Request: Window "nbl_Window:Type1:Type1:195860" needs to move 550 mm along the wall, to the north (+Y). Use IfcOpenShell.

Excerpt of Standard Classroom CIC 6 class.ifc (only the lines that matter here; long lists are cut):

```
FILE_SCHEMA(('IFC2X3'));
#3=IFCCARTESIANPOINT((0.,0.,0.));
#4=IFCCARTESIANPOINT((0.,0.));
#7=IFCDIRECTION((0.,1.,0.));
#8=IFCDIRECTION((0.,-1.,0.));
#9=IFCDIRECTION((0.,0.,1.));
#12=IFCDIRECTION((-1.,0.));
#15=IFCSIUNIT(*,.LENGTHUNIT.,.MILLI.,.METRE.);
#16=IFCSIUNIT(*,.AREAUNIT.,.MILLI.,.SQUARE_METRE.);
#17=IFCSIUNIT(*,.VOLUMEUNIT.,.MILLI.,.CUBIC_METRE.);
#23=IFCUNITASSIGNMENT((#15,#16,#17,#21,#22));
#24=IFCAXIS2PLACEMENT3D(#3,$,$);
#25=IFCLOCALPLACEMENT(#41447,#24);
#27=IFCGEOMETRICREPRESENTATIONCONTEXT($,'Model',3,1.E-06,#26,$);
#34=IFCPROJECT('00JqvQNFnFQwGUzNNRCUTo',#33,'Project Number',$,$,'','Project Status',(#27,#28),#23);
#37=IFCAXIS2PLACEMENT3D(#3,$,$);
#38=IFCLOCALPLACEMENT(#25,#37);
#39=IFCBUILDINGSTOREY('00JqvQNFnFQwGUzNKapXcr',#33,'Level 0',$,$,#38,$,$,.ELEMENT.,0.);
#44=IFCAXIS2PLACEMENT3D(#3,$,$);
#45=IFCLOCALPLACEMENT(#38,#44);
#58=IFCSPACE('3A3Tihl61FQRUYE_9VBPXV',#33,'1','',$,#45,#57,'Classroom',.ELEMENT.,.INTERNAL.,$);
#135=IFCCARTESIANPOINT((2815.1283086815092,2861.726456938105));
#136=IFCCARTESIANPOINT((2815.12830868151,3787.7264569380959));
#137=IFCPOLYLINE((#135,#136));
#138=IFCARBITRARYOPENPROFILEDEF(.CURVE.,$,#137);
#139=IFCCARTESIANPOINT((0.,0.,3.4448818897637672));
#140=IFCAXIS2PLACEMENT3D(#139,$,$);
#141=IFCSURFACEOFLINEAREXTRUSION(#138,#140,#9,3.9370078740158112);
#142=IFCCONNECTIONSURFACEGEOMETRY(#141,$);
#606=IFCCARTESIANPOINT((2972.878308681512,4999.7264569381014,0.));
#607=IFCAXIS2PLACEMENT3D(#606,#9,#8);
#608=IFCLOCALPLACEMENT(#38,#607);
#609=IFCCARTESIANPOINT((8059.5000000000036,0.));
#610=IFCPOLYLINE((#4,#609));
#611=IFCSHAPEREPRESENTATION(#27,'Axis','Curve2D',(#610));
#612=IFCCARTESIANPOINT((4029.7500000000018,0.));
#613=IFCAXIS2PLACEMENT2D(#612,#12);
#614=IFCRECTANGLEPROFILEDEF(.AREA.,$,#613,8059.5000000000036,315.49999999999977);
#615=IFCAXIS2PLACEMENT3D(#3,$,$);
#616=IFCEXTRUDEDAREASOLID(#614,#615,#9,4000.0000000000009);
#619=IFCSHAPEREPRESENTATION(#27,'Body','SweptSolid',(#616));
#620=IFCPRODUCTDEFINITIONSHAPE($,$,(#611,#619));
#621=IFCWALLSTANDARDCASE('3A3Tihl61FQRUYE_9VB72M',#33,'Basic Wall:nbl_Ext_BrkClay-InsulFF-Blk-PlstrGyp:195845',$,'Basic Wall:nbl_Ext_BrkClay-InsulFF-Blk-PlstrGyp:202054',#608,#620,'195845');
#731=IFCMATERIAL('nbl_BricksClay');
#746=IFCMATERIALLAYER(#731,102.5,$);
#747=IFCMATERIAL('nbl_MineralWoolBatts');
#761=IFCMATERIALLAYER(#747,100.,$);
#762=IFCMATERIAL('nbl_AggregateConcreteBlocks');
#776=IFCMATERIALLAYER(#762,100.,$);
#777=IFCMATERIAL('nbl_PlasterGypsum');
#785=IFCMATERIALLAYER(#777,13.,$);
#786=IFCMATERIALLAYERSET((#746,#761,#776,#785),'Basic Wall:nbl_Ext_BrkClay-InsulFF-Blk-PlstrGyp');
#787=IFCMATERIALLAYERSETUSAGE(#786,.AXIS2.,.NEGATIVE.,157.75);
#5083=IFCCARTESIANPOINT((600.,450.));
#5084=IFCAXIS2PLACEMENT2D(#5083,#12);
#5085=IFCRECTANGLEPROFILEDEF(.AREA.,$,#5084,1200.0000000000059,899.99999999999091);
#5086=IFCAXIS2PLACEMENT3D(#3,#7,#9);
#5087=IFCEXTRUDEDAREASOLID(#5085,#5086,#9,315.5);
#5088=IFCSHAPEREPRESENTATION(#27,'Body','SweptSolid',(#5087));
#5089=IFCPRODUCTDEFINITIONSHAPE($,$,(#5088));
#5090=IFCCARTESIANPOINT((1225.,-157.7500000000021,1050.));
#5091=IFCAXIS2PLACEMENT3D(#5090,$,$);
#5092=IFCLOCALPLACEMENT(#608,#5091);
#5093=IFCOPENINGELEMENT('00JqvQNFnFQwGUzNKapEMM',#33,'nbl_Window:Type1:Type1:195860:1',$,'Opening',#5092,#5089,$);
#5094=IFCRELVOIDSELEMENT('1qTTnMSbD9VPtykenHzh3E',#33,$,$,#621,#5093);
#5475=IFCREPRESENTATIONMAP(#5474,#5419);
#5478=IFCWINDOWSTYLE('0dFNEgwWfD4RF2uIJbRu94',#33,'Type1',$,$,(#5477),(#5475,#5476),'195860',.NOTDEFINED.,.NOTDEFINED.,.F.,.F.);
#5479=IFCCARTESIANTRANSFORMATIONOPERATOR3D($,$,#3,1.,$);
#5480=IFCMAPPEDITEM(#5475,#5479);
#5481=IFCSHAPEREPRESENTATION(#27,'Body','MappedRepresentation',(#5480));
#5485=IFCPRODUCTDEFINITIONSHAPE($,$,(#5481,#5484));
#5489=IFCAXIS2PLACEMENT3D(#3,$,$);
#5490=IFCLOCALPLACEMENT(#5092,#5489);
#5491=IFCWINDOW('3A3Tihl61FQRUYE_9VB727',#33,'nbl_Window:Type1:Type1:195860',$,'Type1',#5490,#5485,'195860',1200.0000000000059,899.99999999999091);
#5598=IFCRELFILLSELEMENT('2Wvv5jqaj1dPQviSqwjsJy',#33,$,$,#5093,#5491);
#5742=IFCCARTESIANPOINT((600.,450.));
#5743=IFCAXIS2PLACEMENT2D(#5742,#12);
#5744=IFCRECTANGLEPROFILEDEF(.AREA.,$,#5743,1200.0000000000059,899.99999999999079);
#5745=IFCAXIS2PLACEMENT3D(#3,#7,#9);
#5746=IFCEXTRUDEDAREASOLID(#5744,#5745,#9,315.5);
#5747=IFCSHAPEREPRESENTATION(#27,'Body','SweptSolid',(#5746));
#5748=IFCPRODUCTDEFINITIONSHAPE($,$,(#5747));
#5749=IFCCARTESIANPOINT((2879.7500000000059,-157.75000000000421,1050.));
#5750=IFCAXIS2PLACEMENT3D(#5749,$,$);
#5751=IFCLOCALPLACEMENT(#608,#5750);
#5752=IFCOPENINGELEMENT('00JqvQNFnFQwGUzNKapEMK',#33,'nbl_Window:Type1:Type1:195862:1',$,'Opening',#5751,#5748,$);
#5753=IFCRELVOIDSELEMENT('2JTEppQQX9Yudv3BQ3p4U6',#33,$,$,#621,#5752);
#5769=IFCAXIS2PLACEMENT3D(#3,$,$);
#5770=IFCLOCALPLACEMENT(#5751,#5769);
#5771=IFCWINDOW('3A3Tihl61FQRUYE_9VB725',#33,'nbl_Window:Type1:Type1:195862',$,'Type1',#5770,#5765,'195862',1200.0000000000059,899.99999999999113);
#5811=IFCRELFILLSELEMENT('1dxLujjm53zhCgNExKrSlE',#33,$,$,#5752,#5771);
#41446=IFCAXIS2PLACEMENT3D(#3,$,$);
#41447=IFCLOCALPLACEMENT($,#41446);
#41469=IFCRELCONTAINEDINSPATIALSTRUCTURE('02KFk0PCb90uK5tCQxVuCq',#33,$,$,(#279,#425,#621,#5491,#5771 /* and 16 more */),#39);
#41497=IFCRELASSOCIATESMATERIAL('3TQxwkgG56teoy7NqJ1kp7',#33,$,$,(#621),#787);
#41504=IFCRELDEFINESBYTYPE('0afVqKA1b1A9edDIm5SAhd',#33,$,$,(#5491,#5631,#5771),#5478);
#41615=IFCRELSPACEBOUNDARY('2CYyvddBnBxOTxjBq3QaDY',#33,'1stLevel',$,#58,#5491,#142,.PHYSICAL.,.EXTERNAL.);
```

```python
import numpy as np
import ifcopenshell
import ifcopenshell.api.geometry
import ifcopenshell.util.placement
import ifcopenshell.util.unit

model = ifcopenshell.open("Standard Classroom CIC 6 class.ifc")
unit_scale = ifcopenshell.util.unit.calculate_unit_scale(model)

window = model.by_guid("3A3Tihl61FQRUYE_9VB727")
opening = window.FillsVoids[0].RelatingOpeningElement
wall = opening.VoidsElements[0].RelatingBuildingElement

wall_matrix = ifcopenshell.util.placement.get_local_placement(wall.ObjectPlacement)
shift = wall_matrix[:3, 0] * -0.55 / unit_scale
before = ifcopenshell.util.placement.get_local_placement(window.ObjectPlacement)[:3, 3].copy()

# The window is placed relative to its opening, so it follows when the opening moves.
matrix = ifcopenshell.util.placement.get_local_placement(opening.ObjectPlacement)
matrix[:3, 3] += shift
ifcopenshell.api.geometry.edit_object_placement(
    model, product=opening, matrix=matrix, is_si=False, should_transform_children=True
)

# Space boundary surfaces are stored in each space's coordinates; move them too.
for rel in window.ProvidesBoundaries:
    if not rel.ConnectionGeometry:
        continue
    surface = rel.ConnectionGeometry.SurfaceOnRelatingElement
    space_matrix = ifcopenshell.util.placement.get_local_placement(rel.RelatingSpace.ObjectPlacement)
    point = np.array(surface.Position.Location.Coordinates) + space_matrix[:3, :3].T @ shift
    surface.Position = model.createIfcAxis2Placement3D(
        model.createIfcCartesianPoint(point.tolist()), surface.Position.Axis, surface.Position.RefDirection
    )

after = ifcopenshell.util.placement.get_local_placement(window.ObjectPlacement)[:3, 3]
print("window moved by", (after - before).round(3) + 0.0)

model.write("Standard Classroom CIC 6 class_updated.ifc")
```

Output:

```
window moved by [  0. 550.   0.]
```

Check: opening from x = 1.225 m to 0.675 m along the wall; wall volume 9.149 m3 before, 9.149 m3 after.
